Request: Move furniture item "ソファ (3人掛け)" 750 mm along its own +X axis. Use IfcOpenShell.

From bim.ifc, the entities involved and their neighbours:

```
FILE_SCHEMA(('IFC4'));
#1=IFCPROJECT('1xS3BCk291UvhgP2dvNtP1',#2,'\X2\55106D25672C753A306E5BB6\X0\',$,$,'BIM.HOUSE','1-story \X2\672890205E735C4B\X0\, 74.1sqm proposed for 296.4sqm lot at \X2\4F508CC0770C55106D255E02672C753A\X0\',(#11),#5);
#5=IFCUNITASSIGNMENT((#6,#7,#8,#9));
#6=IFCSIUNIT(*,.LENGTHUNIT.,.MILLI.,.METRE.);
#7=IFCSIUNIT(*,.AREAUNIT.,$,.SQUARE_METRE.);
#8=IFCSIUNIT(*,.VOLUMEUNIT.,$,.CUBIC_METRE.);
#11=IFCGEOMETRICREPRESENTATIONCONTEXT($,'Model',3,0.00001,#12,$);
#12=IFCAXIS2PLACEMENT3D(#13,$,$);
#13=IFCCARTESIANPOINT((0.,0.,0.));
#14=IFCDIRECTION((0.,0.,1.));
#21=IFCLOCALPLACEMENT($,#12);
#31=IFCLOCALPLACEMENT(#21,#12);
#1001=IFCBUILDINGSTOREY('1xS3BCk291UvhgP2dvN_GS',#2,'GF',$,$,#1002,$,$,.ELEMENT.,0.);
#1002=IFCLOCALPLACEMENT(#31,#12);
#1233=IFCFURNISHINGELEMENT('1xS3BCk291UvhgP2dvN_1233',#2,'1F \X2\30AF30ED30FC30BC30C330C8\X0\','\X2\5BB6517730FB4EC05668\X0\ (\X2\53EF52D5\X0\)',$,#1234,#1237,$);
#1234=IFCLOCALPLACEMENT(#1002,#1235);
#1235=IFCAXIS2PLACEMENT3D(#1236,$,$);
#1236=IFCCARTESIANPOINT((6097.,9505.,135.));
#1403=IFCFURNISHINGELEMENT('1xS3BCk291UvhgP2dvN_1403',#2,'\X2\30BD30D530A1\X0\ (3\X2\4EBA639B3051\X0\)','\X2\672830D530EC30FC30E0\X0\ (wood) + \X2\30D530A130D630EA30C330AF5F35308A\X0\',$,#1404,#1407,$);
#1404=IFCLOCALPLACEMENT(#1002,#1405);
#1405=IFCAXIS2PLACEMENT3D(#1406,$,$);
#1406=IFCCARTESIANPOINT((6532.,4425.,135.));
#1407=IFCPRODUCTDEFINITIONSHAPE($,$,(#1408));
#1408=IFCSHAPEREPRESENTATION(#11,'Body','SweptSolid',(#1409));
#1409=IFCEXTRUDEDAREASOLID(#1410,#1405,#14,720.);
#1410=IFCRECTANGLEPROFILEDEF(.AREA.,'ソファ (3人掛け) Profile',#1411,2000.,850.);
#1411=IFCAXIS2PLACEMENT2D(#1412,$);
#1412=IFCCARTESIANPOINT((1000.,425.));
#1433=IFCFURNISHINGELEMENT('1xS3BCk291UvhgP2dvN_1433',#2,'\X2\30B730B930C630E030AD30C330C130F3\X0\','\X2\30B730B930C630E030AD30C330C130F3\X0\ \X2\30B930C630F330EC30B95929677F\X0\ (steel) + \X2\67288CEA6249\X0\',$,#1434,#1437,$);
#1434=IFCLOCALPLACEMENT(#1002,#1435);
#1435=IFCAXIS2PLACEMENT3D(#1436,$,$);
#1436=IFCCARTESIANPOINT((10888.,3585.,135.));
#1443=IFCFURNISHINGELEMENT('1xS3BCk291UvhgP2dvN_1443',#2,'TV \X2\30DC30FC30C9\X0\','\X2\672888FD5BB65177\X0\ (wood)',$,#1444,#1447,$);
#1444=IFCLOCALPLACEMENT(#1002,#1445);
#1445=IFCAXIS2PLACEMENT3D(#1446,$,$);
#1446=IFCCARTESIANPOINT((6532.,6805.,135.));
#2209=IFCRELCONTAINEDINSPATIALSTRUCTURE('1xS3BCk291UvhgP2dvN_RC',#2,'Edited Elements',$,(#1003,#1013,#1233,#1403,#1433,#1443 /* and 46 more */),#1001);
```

```python
import ifcopenshell
import ifcopenshell.api.geometry
import ifcopenshell.util.placement

model = ifcopenshell.open("bim.ifc")

item = model.by_guid("1xS3BCk291UvhgP2dvN_1403")
matrix = ifcopenshell.util.placement.get_local_placement(item.ObjectPlacement)
matrix[:3, 3] += matrix[:3, 0] * 750.0
ifcopenshell.api.geometry.edit_object_placement(model, product=item, matrix=matrix, is_si=False)

print(ifcopenshell.util.placement.get_local_placement(item.ObjectPlacement).round(3) + 0.0)

model.write("bim_updated.ifc")
```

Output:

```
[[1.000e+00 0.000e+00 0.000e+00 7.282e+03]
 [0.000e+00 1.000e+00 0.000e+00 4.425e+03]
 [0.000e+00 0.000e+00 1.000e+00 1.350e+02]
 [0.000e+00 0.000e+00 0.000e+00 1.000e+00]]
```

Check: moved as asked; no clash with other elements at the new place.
